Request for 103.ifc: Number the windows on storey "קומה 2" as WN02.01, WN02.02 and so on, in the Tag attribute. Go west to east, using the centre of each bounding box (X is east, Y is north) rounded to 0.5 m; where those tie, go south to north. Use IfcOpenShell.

First a look at what the model holds.

```python
import ifcopenshell
import ifcopenshell.util.element
import ifcopenshell.util.placement

model = ifcopenshell.open("103.ifc")
print(model.schema)
storey = next(s for s in model.by_type("IfcBuildingStorey") if s.Name == "קומה 2")
windows = [e for e in ifcopenshell.util.element.get_decomposition(storey) if e.is_a("IfcWindow")]
for e in sorted(windows, key=lambda e: e.id()):
    origin = ifcopenshell.util.placement.get_local_placement(e.ObjectPlacement)[:3, 3]
    print(e.id(), e.Tag, e.Name, origin.round(2) + 0.0, sep=" | ")
```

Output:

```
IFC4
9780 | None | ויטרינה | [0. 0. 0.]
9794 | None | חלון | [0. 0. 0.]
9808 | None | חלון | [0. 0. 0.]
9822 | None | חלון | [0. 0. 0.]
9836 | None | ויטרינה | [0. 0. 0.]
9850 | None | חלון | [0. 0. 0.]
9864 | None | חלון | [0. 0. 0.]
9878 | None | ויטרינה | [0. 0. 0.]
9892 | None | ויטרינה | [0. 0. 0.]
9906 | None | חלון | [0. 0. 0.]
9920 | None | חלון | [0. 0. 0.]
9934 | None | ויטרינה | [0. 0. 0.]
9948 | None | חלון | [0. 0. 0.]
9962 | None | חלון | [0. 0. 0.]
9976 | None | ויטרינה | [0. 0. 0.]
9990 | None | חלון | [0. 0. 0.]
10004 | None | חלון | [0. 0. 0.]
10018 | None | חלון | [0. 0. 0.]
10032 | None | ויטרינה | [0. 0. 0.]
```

```python
import ifcopenshell
import ifcopenshell.geom
import ifcopenshell.util.element
import ifcopenshell.util.shape

model = ifcopenshell.open("103.ifc")
settings = ifcopenshell.geom.settings()
settings.set("use-world-coords", True)


def centre(element):
    shape = ifcopenshell.geom.create_shape(settings, element)
    return ifcopenshell.util.shape.get_bbox_centroid(shape.geometry)


storey = next(s for s in model.by_type("IfcBuildingStorey") if s.Name == "קומה 2")
windows = [e for e in ifcopenshell.util.element.get_decomposition(storey) if e.is_a("IfcWindow")]

# Insertion points can sit at a corner or the storey origin, so sort by the geometry (in metres).
centres = {e: centre(e) for e in windows}
windows.sort(key=lambda e: (round(centres[e][0] / 0.5), centres[e][1]))

for i, e in enumerate(windows, start=1):
    number = f"WN02.{i:02d}"
    e.Tag = number
    print(e.id(), number)

model.write("103_v2.ifc")
```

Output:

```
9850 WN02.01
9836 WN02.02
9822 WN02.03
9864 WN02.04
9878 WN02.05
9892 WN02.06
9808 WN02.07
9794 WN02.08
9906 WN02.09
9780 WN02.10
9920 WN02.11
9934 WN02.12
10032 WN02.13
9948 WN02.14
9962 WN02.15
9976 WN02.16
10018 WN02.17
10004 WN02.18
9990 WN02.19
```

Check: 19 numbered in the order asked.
